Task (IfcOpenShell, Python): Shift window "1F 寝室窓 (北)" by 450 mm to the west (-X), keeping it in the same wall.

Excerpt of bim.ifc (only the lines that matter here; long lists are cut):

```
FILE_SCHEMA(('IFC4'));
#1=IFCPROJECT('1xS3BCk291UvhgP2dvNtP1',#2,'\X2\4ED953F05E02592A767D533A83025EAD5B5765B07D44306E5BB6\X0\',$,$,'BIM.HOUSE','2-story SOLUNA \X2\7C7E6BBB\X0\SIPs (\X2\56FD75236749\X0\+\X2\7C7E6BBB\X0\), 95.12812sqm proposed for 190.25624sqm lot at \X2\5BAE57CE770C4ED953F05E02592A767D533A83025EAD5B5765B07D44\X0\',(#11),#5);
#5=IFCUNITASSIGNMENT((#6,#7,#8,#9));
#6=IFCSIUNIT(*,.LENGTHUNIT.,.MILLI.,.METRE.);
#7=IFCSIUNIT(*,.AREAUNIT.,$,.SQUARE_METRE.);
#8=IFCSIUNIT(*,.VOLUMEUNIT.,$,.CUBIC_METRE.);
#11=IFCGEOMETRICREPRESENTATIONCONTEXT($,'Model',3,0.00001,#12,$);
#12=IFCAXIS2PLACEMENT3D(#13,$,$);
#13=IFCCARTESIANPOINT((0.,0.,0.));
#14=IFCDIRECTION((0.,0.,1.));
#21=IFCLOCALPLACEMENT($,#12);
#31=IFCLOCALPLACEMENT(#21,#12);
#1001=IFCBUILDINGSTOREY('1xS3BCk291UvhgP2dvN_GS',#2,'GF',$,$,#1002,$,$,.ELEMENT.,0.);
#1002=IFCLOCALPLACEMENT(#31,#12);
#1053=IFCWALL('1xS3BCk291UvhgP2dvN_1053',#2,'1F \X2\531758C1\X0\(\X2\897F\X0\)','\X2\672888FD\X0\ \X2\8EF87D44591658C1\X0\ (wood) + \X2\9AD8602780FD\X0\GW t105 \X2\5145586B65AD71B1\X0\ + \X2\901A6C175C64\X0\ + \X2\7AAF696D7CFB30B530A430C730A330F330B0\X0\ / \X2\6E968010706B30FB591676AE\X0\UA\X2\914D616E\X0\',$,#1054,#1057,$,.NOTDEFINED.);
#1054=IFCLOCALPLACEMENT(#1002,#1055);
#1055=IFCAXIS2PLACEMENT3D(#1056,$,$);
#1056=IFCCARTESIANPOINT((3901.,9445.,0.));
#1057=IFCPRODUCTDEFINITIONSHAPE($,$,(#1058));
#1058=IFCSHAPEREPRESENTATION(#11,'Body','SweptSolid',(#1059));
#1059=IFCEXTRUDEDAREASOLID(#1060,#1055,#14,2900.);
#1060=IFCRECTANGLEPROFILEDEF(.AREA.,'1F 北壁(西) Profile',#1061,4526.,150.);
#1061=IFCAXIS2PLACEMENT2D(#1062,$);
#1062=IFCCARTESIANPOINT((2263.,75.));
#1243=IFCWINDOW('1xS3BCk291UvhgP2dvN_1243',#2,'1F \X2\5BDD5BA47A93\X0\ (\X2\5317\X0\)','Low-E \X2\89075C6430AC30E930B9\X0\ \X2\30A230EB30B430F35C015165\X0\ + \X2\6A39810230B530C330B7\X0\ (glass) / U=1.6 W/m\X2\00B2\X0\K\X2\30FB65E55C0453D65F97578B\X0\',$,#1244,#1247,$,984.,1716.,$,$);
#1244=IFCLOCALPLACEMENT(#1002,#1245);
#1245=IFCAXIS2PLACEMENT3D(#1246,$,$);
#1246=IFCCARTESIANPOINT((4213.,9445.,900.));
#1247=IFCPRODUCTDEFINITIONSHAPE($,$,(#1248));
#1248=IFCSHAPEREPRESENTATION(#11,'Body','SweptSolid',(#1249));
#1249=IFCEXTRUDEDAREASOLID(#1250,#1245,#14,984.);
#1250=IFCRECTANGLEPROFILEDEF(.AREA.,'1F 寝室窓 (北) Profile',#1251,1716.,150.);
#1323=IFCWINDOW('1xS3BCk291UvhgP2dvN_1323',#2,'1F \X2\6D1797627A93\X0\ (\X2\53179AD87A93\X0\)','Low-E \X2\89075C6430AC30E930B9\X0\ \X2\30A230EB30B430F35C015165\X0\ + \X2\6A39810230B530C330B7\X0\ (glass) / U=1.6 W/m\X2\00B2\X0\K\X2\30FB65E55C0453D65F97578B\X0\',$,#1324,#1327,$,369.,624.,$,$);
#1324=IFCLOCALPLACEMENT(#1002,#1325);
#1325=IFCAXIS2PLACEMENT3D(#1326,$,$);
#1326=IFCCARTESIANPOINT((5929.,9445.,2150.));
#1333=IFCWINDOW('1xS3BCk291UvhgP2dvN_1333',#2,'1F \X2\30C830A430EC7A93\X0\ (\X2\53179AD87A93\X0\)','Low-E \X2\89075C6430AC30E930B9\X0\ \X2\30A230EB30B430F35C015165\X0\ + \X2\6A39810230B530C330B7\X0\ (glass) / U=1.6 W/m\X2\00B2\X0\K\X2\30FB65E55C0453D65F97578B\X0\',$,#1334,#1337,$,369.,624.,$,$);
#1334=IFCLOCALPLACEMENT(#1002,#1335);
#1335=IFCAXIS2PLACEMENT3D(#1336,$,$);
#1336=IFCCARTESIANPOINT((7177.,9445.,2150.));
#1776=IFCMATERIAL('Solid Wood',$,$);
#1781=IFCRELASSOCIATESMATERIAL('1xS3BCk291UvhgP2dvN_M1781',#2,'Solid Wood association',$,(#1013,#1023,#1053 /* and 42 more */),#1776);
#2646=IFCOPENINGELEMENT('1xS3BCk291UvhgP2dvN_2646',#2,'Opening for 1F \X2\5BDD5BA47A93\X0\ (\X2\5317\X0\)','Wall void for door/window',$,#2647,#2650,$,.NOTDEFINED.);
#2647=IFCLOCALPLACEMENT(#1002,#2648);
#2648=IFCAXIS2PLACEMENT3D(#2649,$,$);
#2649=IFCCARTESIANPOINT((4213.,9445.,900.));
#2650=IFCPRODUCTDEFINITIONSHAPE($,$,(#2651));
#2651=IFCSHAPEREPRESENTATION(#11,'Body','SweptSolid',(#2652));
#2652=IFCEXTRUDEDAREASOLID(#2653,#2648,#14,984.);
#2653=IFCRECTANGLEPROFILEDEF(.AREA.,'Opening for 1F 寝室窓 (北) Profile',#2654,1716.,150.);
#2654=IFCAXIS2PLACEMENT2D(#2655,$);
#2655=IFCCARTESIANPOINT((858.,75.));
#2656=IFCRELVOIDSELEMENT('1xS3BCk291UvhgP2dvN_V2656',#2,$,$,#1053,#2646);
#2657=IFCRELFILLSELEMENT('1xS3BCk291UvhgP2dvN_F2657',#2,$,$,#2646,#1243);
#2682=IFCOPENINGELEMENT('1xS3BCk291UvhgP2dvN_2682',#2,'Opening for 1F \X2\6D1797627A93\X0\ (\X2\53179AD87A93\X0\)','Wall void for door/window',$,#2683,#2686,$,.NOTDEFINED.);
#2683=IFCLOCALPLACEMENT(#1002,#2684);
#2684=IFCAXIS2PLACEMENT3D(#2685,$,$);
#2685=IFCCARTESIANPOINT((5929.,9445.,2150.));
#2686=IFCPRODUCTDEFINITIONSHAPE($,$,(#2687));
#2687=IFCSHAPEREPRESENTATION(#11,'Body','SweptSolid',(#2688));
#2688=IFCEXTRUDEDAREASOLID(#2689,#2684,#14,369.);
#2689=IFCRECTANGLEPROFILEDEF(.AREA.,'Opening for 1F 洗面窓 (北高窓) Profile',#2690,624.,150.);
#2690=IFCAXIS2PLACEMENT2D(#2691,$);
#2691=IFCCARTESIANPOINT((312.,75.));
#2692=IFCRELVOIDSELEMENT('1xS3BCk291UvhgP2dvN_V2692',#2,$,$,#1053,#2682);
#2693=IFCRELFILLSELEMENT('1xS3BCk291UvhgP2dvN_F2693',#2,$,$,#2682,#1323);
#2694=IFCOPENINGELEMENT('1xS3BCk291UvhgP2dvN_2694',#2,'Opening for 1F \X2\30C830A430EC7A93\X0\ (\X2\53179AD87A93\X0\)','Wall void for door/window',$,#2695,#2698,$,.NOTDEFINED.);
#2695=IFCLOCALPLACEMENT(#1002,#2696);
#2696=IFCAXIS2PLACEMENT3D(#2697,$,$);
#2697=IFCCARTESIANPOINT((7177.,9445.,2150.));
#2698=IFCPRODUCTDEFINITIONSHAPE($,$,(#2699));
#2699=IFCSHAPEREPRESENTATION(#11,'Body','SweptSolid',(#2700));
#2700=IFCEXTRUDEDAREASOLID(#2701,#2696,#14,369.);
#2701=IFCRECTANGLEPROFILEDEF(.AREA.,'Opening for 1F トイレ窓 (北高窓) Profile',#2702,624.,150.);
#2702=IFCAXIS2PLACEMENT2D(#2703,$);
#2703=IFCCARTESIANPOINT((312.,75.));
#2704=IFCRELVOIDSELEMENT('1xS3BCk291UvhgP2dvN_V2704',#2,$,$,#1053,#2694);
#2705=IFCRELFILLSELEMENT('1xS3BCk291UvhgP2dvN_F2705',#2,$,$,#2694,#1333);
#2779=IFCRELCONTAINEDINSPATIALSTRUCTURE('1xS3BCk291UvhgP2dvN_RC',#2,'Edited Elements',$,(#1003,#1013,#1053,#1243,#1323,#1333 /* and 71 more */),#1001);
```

```python
import ifcopenshell
import ifcopenshell.api.geometry
import ifcopenshell.util.placement
import ifcopenshell.util.unit

model = ifcopenshell.open("bim.ifc")
unit_scale = ifcopenshell.util.unit.calculate_unit_scale(model)

window = model.by_guid("1xS3BCk291UvhgP2dvN_1243")
opening = window.FillsVoids[0].RelatingOpeningElement
wall = opening.VoidsElements[0].RelatingBuildingElement

wall_matrix = ifcopenshell.util.placement.get_local_placement(wall.ObjectPlacement)
shift = wall_matrix[:3, 0] * -0.45 / unit_scale
before = ifcopenshell.util.placement.get_local_placement(window.ObjectPlacement)[:3, 3].copy()

# The window is not placed relative to its opening, so move both.
for product in (opening, window):
    matrix = ifcopenshell.util.placement.get_local_placement(product.ObjectPlacement)
    matrix[:3, 3] += shift
    ifcopenshell.api.geometry.edit_object_placement(model, product=product, matrix=matrix, is_si=False)

after = ifcopenshell.util.placement.get_local_placement(window.ObjectPlacement)[:3, 3]
print("window moved by", (after - before).round(3) + 0.0)

model.write("bim_rev.ifc")
```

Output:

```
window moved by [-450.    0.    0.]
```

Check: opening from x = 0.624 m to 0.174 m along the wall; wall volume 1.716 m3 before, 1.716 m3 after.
